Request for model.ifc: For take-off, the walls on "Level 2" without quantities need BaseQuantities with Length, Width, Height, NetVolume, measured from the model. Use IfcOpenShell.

First a look at what the model holds.

```python
import ifcopenshell
import ifcopenshell.util.element
import ifcopenshell.util.unit

model = ifcopenshell.open("model.ifc")
print(model.schema)
for unit_type in ("LENGTHUNIT", "AREAUNIT", "VOLUMEUNIT"):
    print(unit_type, ifcopenshell.util.unit.calculate_unit_scale(model, unit_type))
storey = next(s for s in model.by_type("IfcBuildingStorey") if s.Name == "Level 2")
walls = [e for e in ifcopenshell.util.element.get_decomposition(storey) if e.is_a("IfcWall")]
for e in sorted(walls, key=lambda e: e.id()):
    print(e.id(), e.is_a(), e.Name, list(ifcopenshell.util.element.get_psets(e, qtos_only=True)), sep=" | ")
```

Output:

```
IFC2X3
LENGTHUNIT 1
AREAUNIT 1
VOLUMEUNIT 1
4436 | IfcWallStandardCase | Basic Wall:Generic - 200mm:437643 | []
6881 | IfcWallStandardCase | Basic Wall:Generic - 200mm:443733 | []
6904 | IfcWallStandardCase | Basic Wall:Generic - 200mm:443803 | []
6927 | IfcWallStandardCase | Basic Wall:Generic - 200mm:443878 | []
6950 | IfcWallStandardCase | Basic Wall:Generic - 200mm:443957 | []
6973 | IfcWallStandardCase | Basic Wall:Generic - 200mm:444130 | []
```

```python
import ifcopenshell
import ifcopenshell.api.pset
import ifcopenshell.geom
import ifcopenshell.util.element
import ifcopenshell.util.shape
import ifcopenshell.util.unit

model = ifcopenshell.open("model.ifc")
unit_scale = ifcopenshell.util.unit.calculate_unit_scale(model)
volume_scale = ifcopenshell.util.unit.calculate_unit_scale(model, "VOLUMEUNIT")
settings = ifcopenshell.geom.settings()

storey = next(s for s in model.by_type("IfcBuildingStorey") if s.Name == "Level 2")
walls = [e for e in ifcopenshell.util.element.get_decomposition(storey) if e.is_a("IfcWall")]

for e in sorted(walls, key=lambda e: e.id()):
    if ifcopenshell.util.element.get_psets(e, qtos_only=True, should_inherit=False):
        continue
    # Geometry comes back in metres, in the element's own axes.
    shape = ifcopenshell.geom.create_shape(settings, e)
    values = {
        "Length": ifcopenshell.util.shape.get_x(shape.geometry) / unit_scale,
        "Width": ifcopenshell.util.shape.get_y(shape.geometry) / unit_scale,
        "Height": ifcopenshell.util.shape.get_z(shape.geometry) / unit_scale,
        "NetVolume": ifcopenshell.util.shape.get_volume(shape.geometry) / volume_scale,
    }
    qto = ifcopenshell.api.pset.add_qto(model, product=e, name="BaseQuantities")
    ifcopenshell.api.pset.edit_qto(model, qto=qto, properties=values)
    print(e.id(), {k: round(v, 3) for k, v in values.items()})

model.write("model-out.ifc")
```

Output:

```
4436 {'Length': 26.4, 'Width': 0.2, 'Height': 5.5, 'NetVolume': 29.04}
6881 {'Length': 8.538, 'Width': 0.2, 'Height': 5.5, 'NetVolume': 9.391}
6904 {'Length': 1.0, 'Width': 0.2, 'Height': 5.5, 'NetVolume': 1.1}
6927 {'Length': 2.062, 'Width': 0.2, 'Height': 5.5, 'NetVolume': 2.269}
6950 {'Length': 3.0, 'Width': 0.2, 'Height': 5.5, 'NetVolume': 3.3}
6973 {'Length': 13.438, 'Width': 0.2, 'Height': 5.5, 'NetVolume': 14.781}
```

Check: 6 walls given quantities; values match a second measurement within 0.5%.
